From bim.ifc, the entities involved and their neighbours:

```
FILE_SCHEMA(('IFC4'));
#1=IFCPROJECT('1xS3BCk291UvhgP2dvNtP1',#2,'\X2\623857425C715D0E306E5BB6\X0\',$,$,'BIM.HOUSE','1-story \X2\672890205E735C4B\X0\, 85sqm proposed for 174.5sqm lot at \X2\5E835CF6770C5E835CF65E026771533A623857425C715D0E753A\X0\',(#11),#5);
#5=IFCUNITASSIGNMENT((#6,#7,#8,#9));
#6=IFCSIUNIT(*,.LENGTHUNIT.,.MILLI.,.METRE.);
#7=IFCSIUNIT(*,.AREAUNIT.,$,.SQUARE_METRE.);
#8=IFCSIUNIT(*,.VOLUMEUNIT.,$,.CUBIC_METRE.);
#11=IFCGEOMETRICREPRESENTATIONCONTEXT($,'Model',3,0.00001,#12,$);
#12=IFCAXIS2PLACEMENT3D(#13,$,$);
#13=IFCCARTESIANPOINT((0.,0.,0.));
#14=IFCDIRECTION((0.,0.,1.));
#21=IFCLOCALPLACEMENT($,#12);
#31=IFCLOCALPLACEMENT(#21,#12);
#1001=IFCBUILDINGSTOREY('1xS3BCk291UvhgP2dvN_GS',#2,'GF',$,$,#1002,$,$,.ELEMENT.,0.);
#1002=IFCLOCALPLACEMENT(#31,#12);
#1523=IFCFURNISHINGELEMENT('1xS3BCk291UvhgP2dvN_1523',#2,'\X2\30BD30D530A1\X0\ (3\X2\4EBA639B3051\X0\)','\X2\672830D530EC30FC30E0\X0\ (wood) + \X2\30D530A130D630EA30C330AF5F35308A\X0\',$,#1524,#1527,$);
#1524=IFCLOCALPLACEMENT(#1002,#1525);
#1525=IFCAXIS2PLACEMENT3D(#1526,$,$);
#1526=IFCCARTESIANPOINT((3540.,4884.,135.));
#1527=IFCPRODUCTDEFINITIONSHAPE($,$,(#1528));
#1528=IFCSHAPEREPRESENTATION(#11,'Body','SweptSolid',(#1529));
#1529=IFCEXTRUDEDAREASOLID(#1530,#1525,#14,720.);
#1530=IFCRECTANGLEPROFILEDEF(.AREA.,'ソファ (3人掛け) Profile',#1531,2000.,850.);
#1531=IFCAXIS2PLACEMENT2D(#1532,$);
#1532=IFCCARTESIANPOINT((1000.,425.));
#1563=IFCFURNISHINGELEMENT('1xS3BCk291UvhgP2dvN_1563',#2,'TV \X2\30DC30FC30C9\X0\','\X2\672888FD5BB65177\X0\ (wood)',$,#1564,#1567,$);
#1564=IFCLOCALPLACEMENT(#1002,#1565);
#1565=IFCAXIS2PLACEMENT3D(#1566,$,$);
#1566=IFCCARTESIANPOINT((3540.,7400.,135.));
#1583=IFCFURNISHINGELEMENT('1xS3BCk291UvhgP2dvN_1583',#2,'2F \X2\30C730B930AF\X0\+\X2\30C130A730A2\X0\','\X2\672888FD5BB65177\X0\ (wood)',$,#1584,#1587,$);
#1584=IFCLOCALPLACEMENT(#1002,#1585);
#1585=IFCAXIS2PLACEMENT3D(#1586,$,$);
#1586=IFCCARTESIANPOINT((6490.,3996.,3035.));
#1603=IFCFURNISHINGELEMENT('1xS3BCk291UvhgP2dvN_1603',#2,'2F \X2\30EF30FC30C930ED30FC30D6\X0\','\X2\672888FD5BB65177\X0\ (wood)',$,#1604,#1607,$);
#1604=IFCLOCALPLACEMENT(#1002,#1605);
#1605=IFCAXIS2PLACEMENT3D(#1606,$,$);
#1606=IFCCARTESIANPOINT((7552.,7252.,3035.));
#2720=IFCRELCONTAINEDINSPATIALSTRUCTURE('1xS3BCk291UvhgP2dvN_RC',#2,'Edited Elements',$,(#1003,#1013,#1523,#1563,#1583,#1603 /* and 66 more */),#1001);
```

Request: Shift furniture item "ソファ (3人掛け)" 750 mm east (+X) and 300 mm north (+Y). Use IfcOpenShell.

```python
import ifcopenshell
import ifcopenshell.api.geometry
import ifcopenshell.util.placement
import ifcopenshell.util.unit

model = ifcopenshell.open("bim.ifc")
unit_scale = ifcopenshell.util.unit.calculate_unit_scale(model)

item = model.by_id(1523)
matrix = ifcopenshell.util.placement.get_local_placement(item.ObjectPlacement)
matrix[0, 3] += 0.75 / unit_scale
matrix[1, 3] += 0.3 / unit_scale
ifcopenshell.api.geometry.edit_object_placement(model, product=item, matrix=matrix, is_si=False)

print(ifcopenshell.util.placement.get_local_placement(item.ObjectPlacement).round(3) + 0.0)

model.write("bim_v2.ifc")
```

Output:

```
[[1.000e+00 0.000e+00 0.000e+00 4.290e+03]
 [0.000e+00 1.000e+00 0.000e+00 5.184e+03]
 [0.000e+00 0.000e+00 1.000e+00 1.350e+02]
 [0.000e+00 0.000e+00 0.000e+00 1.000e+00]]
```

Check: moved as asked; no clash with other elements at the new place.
